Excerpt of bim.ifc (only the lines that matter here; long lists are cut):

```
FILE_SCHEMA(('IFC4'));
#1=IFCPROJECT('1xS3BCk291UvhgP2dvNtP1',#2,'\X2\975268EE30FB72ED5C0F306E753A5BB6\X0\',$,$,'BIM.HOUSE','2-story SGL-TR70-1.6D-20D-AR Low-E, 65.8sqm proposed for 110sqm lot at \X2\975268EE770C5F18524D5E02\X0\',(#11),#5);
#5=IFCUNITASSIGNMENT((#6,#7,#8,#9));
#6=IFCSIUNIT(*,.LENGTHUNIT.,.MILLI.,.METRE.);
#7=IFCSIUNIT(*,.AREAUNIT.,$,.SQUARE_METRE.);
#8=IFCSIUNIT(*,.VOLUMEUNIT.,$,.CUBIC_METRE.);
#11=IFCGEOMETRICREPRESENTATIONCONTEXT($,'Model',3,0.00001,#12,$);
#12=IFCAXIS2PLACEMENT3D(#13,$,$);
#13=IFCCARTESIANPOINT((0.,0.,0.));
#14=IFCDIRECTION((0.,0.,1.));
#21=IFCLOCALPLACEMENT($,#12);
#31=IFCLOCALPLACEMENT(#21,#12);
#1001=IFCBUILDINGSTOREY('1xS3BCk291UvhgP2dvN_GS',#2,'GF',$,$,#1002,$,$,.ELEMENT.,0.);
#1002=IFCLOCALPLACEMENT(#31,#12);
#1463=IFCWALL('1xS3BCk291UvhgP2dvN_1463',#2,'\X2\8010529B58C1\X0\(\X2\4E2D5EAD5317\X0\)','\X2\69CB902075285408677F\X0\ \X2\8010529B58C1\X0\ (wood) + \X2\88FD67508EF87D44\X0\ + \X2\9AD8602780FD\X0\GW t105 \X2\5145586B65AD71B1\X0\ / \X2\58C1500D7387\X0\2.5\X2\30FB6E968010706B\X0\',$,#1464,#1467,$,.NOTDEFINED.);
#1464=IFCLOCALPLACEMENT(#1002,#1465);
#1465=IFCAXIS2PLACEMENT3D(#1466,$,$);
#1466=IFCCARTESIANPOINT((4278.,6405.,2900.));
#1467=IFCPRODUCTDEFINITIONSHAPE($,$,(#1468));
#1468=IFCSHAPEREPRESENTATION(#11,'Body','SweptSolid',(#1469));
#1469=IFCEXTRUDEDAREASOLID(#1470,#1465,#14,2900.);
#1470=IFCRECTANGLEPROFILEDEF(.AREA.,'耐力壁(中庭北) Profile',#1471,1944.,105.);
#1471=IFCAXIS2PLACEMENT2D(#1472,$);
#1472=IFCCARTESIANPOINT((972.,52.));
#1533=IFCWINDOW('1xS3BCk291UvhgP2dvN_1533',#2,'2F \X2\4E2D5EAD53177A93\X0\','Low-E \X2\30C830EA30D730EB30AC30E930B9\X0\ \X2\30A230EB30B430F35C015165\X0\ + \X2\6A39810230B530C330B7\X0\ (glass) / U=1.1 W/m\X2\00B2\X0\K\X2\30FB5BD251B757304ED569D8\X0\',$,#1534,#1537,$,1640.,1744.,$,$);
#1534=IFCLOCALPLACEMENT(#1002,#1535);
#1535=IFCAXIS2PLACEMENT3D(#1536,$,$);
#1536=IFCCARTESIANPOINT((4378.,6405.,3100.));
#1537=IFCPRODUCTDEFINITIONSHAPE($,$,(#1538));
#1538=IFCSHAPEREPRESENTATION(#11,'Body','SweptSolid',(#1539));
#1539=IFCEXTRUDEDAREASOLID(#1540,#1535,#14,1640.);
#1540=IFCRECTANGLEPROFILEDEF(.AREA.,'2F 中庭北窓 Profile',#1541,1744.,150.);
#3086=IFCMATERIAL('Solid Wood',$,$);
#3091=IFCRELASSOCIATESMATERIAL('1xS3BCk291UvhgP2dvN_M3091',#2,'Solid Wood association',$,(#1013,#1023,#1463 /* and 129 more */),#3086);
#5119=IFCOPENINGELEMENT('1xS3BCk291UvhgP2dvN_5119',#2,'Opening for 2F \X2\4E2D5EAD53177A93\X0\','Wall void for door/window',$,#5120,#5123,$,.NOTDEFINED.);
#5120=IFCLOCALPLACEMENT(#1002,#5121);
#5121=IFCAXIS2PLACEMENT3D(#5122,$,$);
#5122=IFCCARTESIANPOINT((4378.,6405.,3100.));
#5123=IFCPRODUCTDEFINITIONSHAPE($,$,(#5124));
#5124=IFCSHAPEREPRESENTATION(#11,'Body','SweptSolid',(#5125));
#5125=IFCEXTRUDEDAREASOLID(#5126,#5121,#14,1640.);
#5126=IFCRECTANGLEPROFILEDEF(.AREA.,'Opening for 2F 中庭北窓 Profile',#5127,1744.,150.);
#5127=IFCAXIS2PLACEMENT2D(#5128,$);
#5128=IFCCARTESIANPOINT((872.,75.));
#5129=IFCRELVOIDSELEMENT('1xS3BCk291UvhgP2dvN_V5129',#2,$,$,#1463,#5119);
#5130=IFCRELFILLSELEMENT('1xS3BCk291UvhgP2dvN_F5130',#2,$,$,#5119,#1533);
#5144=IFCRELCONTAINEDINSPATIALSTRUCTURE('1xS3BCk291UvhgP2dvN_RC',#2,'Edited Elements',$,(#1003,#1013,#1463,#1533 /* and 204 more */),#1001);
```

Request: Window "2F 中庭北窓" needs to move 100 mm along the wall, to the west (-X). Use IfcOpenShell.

```python
import ifcopenshell
import ifcopenshell.api.geometry
import ifcopenshell.util.placement

model = ifcopenshell.open("bim.ifc")

window = model.by_guid("1xS3BCk291UvhgP2dvN_1533")
opening = window.FillsVoids[0].RelatingOpeningElement
wall = opening.VoidsElements[0].RelatingBuildingElement

wall_matrix = ifcopenshell.util.placement.get_local_placement(wall.ObjectPlacement)
shift = wall_matrix[:3, 0] * -100.0
before = ifcopenshell.util.placement.get_local_placement(window.ObjectPlacement)[:3, 3].copy()

# The window is not placed relative to its opening, so move both.
for product in (opening, window):
    matrix = ifcopenshell.util.placement.get_local_placement(product.ObjectPlacement)
    matrix[:3, 3] += shift
    ifcopenshell.api.geometry.edit_object_placement(model, product=product, matrix=matrix, is_si=False)

after = ifcopenshell.util.placement.get_local_placement(window.ObjectPlacement)[:3, 3]
print("window moved by", (after - before).round(3) + 0.0)

model.write("bim_updated.ifc")
```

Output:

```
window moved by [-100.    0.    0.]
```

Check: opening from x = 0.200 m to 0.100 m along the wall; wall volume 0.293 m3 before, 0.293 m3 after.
